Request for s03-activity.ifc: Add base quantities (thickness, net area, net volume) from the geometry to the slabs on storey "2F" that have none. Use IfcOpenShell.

First a look at what the model holds.

```python
import ifcopenshell
import ifcopenshell.util.element
import ifcopenshell.util.unit

model = ifcopenshell.open("s03-activity.ifc")
print(model.schema)
for unit_type in ("LENGTHUNIT", "AREAUNIT", "VOLUMEUNIT"):
    print(unit_type, ifcopenshell.util.unit.calculate_unit_scale(model, unit_type))
storey = next(s for s in model.by_type("IfcBuildingStorey") if s.Name == "2F")
slabs = [e for e in ifcopenshell.util.element.get_decomposition(storey) if e.is_a("IfcSlab")]
for e in sorted(slabs, key=lambda e: e.id()):
    print(e.id(), e.is_a(), e.Name, list(ifcopenshell.util.element.get_psets(e, qtos_only=True)), sep=" | ")
```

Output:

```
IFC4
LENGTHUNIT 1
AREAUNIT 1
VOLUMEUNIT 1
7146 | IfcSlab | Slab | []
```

```python
import ifcopenshell
import ifcopenshell.api.pset
import ifcopenshell.geom
import ifcopenshell.util.element
import ifcopenshell.util.shape
import ifcopenshell.util.unit

model = ifcopenshell.open("s03-activity.ifc")
unit_scale = ifcopenshell.util.unit.calculate_unit_scale(model)
area_scale = ifcopenshell.util.unit.calculate_unit_scale(model, "AREAUNIT")
volume_scale = ifcopenshell.util.unit.calculate_unit_scale(model, "VOLUMEUNIT")
settings = ifcopenshell.geom.settings()

storey = next(s for s in model.by_type("IfcBuildingStorey") if s.Name == "2F")
slabs = [e for e in ifcopenshell.util.element.get_decomposition(storey) if e.is_a("IfcSlab")]

for e in sorted(slabs, key=lambda e: e.id()):
    if ifcopenshell.util.element.get_psets(e, qtos_only=True, should_inherit=False):
        continue
    # Geometry comes back in metres, in the element's own axes.
    shape = ifcopenshell.geom.create_shape(settings, e)
    values = {
        "Width": ifcopenshell.util.shape.get_z(shape.geometry) / unit_scale,
        "NetArea": ifcopenshell.util.shape.get_footprint_area(shape.geometry) / area_scale,
        "NetVolume": ifcopenshell.util.shape.get_volume(shape.geometry) / volume_scale,
    }
    qto = ifcopenshell.api.pset.add_qto(model, product=e, name="Qto_SlabBaseQuantities")
    ifcopenshell.api.pset.edit_qto(model, qto=qto, properties=values)
    print(e.id(), {k: round(v, 3) for k, v in values.items()})

model.write("s03-activity-out.ifc")
```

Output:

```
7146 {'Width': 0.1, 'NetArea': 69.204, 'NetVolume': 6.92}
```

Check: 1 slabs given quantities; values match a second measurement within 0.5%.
